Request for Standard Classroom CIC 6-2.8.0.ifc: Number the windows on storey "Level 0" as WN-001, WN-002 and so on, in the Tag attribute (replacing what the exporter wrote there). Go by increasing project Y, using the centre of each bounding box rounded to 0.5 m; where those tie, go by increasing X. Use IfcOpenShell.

First a look at what the model holds.

```python
import ifcopenshell
import ifcopenshell.util.element
import ifcopenshell.util.placement

model = ifcopenshell.open("Standard Classroom CIC 6-2.8.0.ifc")
print(model.schema)
storey = next(s for s in model.by_type("IfcBuildingStorey") if s.Name == "Level 0")
windows = [e for e in ifcopenshell.util.element.get_decomposition(storey) if e.is_a("IfcWindow")]
for e in sorted(windows, key=lambda e: e.id()):
    origin = ifcopenshell.util.placement.get_local_placement(e.ObjectPlacement)[:3, 3]
    print(e.id(), e.Tag, e.Name, origin.round(2) + 0.0, sep=" | ")
```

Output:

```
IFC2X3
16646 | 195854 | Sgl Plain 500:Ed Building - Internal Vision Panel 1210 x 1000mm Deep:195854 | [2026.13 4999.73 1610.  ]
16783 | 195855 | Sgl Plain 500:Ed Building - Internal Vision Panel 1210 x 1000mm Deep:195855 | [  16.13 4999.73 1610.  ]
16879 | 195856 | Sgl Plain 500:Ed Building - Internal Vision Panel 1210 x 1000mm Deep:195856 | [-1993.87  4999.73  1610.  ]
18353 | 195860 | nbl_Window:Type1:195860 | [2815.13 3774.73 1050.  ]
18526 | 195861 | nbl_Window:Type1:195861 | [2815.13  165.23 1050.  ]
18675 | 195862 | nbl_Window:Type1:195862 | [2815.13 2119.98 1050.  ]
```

```python
import ifcopenshell
import ifcopenshell.geom
import ifcopenshell.util.element
import ifcopenshell.util.shape

model = ifcopenshell.open("Standard Classroom CIC 6-2.8.0.ifc")
settings = ifcopenshell.geom.settings()
settings.set("use-world-coords", True)


def centre(element):
    shape = ifcopenshell.geom.create_shape(settings, element)
    return ifcopenshell.util.shape.get_bbox_centroid(shape.geometry)


storey = next(s for s in model.by_type("IfcBuildingStorey") if s.Name == "Level 0")
windows = [e for e in ifcopenshell.util.element.get_decomposition(storey) if e.is_a("IfcWindow")]

# Insertion points can sit at a corner or the storey origin, so sort by the geometry (in metres).
centres = {e: centre(e) for e in windows}
windows.sort(key=lambda e: (round(centres[e][1] / 0.5), centres[e][0]))

for i, e in enumerate(windows, start=1):
    number = f"WN-0{i:02d}"
    e.Tag = number
    print(e.id(), number)

model.write("Standard Classroom CIC 6-2.8.0_v2.ifc")
```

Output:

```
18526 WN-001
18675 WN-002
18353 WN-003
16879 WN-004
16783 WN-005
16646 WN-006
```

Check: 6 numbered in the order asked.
